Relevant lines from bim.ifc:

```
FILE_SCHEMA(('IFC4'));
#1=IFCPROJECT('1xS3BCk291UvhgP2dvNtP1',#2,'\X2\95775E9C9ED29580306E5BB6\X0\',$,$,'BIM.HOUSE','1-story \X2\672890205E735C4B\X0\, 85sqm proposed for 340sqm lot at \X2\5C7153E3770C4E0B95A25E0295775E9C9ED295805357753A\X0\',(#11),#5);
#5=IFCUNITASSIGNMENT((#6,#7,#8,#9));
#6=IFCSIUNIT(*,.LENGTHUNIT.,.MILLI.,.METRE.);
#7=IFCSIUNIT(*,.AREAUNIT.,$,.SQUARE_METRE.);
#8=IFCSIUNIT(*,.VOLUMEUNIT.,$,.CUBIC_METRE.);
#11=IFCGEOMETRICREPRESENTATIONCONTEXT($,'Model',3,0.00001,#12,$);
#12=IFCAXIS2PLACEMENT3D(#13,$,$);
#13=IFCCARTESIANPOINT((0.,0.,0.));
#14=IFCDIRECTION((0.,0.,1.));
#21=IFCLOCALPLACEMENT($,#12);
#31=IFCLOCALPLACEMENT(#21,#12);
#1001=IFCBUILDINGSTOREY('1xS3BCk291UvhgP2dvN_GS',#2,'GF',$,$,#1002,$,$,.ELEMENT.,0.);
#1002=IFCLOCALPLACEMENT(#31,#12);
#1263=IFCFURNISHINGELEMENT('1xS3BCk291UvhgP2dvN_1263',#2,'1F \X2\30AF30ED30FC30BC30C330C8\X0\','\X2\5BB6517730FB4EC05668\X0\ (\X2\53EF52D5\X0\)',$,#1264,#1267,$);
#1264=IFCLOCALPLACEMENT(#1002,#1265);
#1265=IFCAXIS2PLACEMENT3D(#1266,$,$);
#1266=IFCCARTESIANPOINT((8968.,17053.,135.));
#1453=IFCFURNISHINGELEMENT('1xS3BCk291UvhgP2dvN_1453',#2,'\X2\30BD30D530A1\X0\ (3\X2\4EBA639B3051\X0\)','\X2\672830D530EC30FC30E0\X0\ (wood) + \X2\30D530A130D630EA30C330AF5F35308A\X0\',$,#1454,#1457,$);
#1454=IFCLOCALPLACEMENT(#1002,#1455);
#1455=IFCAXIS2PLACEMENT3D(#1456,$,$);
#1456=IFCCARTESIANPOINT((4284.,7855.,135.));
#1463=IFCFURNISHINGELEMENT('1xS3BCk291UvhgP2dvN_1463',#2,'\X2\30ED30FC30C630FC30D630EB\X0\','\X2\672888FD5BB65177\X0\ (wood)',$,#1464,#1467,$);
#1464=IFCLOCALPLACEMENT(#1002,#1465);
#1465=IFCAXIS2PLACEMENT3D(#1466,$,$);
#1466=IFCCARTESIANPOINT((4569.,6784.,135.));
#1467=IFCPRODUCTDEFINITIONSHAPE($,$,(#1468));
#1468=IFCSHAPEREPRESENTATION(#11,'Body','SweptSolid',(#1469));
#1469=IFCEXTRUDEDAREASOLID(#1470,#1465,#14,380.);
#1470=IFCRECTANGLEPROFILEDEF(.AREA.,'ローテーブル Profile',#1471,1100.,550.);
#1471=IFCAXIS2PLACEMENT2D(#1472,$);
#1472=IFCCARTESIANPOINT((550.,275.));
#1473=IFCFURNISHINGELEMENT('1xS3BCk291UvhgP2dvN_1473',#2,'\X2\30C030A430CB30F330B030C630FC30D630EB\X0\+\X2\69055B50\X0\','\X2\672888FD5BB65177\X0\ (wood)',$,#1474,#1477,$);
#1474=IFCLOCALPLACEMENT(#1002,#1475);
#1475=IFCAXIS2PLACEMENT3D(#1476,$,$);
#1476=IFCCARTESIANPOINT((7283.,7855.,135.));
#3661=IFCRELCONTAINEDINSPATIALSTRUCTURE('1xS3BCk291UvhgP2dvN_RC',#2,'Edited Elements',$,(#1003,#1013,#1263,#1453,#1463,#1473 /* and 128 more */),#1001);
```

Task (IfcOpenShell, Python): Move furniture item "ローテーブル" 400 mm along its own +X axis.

```python
import ifcopenshell
import ifcopenshell.api.geometry
import ifcopenshell.util.placement
import ifcopenshell.util.unit

model = ifcopenshell.open("bim.ifc")
unit_scale = ifcopenshell.util.unit.calculate_unit_scale(model)

item = model.by_id(1463)
matrix = ifcopenshell.util.placement.get_local_placement(item.ObjectPlacement)
matrix[:3, 3] += matrix[:3, 0] * 0.4 / unit_scale
ifcopenshell.api.geometry.edit_object_placement(model, product=item, matrix=matrix, is_si=False)

print(ifcopenshell.util.placement.get_local_placement(item.ObjectPlacement).round(3) + 0.0)

model.write("bim_edited.ifc")
```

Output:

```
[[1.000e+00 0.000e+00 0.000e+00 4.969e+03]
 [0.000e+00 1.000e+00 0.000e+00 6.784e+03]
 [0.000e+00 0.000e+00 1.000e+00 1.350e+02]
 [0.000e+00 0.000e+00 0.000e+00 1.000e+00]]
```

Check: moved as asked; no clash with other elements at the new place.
